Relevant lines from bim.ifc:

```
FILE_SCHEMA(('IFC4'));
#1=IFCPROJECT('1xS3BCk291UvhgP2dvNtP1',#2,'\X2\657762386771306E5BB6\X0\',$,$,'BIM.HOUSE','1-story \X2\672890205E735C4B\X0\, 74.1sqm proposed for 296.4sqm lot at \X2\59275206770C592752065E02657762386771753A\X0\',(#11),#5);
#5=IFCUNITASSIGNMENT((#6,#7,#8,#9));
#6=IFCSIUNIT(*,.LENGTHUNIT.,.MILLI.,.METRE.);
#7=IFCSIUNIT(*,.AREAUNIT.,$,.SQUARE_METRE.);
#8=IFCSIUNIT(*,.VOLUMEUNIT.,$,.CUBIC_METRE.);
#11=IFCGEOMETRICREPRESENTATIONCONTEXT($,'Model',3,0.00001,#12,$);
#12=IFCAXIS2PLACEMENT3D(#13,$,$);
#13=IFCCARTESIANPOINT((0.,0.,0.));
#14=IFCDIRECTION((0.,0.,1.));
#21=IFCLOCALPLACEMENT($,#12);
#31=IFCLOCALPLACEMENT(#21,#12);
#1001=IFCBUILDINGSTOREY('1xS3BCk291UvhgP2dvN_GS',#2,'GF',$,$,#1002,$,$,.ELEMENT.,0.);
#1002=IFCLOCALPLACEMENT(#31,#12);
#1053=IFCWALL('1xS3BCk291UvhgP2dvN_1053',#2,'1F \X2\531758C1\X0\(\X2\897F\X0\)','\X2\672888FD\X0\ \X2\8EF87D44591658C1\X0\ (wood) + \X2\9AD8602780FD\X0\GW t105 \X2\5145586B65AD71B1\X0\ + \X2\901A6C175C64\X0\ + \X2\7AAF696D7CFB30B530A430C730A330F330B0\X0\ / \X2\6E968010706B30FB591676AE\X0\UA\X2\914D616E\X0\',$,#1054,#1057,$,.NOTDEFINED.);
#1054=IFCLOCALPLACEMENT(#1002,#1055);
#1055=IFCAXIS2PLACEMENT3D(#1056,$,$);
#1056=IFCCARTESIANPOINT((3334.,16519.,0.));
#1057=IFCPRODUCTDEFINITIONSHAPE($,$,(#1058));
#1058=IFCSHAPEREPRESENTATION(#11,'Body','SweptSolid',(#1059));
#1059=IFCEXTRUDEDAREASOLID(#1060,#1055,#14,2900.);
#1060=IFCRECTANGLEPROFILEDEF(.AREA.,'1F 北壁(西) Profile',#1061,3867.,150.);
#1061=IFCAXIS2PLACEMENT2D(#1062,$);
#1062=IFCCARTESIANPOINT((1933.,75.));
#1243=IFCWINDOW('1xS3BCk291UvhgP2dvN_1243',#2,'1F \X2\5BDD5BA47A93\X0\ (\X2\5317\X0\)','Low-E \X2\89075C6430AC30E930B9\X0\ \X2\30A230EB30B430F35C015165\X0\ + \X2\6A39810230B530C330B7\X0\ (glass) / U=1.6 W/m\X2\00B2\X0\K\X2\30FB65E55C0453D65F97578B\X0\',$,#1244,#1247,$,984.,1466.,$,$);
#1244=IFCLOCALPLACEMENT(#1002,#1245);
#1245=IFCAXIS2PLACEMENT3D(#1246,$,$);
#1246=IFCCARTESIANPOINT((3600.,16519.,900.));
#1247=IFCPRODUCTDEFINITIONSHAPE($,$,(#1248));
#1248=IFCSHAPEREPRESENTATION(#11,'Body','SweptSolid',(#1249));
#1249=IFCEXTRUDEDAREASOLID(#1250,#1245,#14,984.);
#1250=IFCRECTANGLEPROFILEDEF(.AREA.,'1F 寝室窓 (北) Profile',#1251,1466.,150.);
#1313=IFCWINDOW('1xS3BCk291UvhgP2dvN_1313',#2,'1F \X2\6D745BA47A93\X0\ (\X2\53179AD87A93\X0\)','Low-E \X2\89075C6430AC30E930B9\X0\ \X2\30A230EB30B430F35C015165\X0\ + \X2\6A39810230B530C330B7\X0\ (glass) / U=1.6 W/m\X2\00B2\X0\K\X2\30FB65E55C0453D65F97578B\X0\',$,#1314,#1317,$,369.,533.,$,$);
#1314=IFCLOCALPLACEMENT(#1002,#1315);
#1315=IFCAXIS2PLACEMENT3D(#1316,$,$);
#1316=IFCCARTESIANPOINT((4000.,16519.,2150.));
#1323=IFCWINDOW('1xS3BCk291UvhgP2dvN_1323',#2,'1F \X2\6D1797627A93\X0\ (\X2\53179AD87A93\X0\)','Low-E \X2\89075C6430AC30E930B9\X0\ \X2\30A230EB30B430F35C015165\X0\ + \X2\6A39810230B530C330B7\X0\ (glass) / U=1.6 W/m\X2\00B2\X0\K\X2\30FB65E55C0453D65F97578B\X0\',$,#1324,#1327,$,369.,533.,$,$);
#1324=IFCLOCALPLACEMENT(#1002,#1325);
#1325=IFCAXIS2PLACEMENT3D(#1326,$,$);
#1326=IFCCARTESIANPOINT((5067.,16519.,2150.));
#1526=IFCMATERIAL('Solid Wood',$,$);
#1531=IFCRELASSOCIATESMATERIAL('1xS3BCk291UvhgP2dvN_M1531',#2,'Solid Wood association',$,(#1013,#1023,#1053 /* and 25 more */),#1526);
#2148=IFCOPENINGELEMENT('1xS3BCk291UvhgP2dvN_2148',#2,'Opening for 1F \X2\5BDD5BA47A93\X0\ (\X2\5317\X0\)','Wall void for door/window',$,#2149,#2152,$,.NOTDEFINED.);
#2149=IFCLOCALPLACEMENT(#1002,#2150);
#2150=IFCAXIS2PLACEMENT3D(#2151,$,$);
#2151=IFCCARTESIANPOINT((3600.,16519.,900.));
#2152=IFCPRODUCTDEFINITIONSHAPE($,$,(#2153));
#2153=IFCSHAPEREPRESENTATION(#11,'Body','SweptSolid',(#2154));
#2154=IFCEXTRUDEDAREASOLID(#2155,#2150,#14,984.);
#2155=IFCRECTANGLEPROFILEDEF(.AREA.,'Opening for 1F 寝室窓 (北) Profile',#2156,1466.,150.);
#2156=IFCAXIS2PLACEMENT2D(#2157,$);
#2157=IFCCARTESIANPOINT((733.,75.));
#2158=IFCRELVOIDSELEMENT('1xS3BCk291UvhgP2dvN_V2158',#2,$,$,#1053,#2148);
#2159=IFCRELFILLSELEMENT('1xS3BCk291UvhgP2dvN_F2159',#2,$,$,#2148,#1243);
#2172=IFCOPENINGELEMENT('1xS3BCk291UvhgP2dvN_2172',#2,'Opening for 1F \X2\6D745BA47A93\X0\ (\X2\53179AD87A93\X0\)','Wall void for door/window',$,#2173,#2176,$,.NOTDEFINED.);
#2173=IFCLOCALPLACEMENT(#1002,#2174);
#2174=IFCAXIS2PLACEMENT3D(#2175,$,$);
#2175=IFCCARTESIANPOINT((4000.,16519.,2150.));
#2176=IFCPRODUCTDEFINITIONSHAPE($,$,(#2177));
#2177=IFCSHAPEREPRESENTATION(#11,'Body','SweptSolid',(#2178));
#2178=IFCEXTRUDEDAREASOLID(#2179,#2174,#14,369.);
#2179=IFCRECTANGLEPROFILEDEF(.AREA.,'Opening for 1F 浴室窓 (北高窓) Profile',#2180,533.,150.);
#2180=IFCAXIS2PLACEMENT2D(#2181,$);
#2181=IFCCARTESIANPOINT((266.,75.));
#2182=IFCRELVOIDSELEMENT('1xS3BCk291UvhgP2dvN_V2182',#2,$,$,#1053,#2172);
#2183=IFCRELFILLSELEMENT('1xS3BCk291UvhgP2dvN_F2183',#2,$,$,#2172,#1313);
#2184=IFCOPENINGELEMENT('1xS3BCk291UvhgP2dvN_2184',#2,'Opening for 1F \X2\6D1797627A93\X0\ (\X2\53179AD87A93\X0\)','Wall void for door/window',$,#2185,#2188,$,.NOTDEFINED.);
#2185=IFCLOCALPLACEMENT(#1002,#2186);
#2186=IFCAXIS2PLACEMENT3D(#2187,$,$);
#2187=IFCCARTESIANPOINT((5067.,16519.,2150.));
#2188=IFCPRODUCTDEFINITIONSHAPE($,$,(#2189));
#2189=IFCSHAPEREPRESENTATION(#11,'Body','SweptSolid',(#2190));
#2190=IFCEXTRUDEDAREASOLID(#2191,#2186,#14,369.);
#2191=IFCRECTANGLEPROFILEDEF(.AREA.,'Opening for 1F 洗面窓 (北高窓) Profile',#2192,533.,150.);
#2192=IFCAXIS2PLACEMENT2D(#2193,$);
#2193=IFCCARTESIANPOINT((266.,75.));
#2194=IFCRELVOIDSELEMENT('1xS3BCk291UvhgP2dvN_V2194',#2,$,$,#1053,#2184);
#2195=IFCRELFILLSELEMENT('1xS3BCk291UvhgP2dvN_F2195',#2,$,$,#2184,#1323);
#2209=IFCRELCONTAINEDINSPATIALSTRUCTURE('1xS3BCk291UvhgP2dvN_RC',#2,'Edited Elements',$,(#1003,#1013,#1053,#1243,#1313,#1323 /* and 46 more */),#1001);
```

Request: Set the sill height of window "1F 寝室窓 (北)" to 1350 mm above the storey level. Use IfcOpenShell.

```python
import numpy as np
import ifcopenshell
import ifcopenshell.api.geometry
import ifcopenshell.geom
import ifcopenshell.util.element
import ifcopenshell.util.placement
import ifcopenshell.util.shape
import ifcopenshell.util.unit

model = ifcopenshell.open("bim.ifc")
unit_scale = ifcopenshell.util.unit.calculate_unit_scale(model)

window = model.by_guid("1xS3BCk291UvhgP2dvN_1243")
opening = window.FillsVoids[0].RelatingOpeningElement
storey = ifcopenshell.util.element.get_container(window, ifc_class="IfcBuildingStorey")
level = ifcopenshell.util.placement.get_local_placement(storey.ObjectPlacement)[2, 3]

# The opening's origin need not be at the sill, so measure its lowest point.
shape = ifcopenshell.geom.create_shape(ifcopenshell.geom.settings(), opening)
bottom = ifcopenshell.util.shape.get_shape_bottom_elevation(shape, shape.geometry) / unit_scale
dz = level + 1.35 / unit_scale - bottom

shift = np.array([0.0, 0.0, dz])
# The window is not placed relative to its opening, so move both.
for product in (opening, window):
    matrix = ifcopenshell.util.placement.get_local_placement(product.ObjectPlacement)
    matrix[:3, 3] += shift
    ifcopenshell.api.geometry.edit_object_placement(model, product=product, matrix=matrix, is_si=False)

print(f"moved by {dz * unit_scale:+.3f} m")

model.write("bim_edited.ifc")
```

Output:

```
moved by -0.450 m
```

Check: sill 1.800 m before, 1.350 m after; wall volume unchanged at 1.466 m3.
